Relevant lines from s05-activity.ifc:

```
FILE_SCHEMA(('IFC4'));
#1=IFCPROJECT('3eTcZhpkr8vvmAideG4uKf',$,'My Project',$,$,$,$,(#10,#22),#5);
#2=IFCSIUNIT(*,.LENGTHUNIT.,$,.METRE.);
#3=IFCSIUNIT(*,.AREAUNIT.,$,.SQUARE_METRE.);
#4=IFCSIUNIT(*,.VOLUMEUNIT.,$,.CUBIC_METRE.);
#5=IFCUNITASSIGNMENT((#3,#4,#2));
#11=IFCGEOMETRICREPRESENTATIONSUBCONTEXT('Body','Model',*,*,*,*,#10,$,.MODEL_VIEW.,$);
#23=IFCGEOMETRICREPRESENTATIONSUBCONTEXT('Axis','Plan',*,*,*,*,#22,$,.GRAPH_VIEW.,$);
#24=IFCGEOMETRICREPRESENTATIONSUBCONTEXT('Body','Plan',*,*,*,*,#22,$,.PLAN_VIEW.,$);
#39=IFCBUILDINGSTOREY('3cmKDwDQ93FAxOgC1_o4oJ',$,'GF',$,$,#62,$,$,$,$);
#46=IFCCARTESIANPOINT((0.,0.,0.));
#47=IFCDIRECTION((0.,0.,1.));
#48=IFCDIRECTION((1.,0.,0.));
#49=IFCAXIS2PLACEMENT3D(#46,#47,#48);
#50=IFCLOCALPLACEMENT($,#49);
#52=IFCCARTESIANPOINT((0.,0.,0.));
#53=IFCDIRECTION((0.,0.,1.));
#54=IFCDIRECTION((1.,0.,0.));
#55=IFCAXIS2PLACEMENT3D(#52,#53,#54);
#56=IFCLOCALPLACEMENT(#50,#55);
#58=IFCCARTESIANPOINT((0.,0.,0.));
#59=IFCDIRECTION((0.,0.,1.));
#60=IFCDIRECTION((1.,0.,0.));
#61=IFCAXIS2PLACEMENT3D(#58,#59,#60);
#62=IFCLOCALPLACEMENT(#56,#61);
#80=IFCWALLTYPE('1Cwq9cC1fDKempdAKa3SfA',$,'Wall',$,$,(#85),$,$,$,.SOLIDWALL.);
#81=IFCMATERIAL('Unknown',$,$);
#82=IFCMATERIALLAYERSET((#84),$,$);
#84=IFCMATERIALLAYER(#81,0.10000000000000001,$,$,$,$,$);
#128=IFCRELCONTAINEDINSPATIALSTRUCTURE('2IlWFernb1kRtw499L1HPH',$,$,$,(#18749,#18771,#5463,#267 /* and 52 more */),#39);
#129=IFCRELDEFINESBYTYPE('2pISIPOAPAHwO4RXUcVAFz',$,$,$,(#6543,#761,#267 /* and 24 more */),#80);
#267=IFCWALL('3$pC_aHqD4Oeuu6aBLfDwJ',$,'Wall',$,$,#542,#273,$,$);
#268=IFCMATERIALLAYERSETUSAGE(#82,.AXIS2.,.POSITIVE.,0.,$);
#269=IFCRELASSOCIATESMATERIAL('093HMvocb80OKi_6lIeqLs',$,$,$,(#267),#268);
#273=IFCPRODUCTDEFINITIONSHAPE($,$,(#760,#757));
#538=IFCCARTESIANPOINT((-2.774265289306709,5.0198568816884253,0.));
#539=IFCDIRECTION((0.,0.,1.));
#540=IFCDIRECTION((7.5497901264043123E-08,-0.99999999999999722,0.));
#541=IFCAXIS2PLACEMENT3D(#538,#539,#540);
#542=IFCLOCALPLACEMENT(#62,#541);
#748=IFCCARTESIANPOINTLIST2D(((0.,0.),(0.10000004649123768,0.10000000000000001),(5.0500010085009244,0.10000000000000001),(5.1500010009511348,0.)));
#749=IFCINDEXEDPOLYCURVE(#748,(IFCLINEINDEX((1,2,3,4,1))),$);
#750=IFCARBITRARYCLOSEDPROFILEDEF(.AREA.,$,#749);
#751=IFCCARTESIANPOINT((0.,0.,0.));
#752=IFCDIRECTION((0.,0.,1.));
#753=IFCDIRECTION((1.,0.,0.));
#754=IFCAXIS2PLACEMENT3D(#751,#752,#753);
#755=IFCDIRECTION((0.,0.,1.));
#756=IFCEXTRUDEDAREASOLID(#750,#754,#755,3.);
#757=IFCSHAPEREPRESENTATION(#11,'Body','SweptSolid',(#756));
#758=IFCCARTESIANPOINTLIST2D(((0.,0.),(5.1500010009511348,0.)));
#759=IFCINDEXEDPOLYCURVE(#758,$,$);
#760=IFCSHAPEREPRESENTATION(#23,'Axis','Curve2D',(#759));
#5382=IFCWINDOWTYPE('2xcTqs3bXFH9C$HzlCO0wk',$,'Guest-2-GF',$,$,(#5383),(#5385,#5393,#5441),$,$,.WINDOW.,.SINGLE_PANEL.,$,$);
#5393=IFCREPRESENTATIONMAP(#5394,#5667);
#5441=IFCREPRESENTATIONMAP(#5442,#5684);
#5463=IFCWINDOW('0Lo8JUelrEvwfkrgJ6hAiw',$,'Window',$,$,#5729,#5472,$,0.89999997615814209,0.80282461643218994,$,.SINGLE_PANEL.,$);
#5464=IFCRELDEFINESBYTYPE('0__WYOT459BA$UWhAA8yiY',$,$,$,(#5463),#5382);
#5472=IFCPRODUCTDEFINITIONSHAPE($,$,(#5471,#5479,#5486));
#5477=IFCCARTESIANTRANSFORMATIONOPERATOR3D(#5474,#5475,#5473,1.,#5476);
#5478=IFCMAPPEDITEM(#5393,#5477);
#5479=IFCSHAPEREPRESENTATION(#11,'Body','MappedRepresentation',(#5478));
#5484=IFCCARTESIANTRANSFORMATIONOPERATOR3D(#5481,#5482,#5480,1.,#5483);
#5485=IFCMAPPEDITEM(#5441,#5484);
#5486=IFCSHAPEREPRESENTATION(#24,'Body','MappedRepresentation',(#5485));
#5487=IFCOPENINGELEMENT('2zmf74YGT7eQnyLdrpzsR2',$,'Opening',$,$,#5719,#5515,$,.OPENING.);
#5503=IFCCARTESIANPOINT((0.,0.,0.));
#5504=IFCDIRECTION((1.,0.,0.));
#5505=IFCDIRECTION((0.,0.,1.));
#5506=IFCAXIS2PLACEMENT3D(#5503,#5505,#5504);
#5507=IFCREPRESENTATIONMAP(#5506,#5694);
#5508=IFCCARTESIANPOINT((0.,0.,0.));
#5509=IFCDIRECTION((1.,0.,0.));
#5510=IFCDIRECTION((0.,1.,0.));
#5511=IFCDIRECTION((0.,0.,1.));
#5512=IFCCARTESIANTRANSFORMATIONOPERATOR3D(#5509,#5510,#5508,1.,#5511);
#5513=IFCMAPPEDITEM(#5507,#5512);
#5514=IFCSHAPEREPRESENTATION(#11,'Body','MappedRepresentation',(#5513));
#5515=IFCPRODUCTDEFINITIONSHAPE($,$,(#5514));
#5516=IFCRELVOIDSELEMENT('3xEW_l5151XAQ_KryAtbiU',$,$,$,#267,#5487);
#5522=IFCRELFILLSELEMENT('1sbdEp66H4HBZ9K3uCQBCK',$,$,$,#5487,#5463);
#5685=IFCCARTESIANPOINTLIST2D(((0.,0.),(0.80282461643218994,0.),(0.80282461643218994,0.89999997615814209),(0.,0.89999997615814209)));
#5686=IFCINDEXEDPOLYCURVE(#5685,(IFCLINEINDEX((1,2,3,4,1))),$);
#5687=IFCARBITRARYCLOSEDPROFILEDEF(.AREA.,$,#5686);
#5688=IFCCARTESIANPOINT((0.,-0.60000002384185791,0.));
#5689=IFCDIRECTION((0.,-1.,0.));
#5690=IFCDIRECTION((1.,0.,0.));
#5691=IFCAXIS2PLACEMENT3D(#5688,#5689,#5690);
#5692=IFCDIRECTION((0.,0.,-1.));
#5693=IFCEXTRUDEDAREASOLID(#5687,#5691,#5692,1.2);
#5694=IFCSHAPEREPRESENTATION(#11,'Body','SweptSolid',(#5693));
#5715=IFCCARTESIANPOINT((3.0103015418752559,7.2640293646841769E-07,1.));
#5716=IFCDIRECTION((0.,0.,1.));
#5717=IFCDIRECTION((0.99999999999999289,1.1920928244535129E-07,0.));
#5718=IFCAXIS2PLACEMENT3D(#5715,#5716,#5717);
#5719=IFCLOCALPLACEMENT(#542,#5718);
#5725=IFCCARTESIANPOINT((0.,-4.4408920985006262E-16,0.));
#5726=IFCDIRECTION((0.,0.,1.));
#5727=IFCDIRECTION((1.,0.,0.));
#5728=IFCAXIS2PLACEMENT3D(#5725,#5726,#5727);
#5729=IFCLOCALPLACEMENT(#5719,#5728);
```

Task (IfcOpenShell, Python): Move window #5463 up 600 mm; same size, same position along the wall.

```python
import numpy as np
import ifcopenshell
import ifcopenshell.api.geometry
import ifcopenshell.util.placement
import ifcopenshell.util.unit

model = ifcopenshell.open("s05-activity.ifc")
unit_scale = ifcopenshell.util.unit.calculate_unit_scale(model)

window = model.by_id(5463)
opening = window.FillsVoids[0].RelatingOpeningElement
dz = 0.6 / unit_scale

shift = np.array([0.0, 0.0, dz])
# The window is placed relative to its opening, so it follows when the opening moves.
matrix = ifcopenshell.util.placement.get_local_placement(opening.ObjectPlacement)
matrix[:3, 3] += shift
ifcopenshell.api.geometry.edit_object_placement(
    model, product=opening, matrix=matrix, is_si=False, should_transform_children=True
)

print(f"moved by {dz * unit_scale:+.3f} m")

model.write("s05-activity-out.ifc")
```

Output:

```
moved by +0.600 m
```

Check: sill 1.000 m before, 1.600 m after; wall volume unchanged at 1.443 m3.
